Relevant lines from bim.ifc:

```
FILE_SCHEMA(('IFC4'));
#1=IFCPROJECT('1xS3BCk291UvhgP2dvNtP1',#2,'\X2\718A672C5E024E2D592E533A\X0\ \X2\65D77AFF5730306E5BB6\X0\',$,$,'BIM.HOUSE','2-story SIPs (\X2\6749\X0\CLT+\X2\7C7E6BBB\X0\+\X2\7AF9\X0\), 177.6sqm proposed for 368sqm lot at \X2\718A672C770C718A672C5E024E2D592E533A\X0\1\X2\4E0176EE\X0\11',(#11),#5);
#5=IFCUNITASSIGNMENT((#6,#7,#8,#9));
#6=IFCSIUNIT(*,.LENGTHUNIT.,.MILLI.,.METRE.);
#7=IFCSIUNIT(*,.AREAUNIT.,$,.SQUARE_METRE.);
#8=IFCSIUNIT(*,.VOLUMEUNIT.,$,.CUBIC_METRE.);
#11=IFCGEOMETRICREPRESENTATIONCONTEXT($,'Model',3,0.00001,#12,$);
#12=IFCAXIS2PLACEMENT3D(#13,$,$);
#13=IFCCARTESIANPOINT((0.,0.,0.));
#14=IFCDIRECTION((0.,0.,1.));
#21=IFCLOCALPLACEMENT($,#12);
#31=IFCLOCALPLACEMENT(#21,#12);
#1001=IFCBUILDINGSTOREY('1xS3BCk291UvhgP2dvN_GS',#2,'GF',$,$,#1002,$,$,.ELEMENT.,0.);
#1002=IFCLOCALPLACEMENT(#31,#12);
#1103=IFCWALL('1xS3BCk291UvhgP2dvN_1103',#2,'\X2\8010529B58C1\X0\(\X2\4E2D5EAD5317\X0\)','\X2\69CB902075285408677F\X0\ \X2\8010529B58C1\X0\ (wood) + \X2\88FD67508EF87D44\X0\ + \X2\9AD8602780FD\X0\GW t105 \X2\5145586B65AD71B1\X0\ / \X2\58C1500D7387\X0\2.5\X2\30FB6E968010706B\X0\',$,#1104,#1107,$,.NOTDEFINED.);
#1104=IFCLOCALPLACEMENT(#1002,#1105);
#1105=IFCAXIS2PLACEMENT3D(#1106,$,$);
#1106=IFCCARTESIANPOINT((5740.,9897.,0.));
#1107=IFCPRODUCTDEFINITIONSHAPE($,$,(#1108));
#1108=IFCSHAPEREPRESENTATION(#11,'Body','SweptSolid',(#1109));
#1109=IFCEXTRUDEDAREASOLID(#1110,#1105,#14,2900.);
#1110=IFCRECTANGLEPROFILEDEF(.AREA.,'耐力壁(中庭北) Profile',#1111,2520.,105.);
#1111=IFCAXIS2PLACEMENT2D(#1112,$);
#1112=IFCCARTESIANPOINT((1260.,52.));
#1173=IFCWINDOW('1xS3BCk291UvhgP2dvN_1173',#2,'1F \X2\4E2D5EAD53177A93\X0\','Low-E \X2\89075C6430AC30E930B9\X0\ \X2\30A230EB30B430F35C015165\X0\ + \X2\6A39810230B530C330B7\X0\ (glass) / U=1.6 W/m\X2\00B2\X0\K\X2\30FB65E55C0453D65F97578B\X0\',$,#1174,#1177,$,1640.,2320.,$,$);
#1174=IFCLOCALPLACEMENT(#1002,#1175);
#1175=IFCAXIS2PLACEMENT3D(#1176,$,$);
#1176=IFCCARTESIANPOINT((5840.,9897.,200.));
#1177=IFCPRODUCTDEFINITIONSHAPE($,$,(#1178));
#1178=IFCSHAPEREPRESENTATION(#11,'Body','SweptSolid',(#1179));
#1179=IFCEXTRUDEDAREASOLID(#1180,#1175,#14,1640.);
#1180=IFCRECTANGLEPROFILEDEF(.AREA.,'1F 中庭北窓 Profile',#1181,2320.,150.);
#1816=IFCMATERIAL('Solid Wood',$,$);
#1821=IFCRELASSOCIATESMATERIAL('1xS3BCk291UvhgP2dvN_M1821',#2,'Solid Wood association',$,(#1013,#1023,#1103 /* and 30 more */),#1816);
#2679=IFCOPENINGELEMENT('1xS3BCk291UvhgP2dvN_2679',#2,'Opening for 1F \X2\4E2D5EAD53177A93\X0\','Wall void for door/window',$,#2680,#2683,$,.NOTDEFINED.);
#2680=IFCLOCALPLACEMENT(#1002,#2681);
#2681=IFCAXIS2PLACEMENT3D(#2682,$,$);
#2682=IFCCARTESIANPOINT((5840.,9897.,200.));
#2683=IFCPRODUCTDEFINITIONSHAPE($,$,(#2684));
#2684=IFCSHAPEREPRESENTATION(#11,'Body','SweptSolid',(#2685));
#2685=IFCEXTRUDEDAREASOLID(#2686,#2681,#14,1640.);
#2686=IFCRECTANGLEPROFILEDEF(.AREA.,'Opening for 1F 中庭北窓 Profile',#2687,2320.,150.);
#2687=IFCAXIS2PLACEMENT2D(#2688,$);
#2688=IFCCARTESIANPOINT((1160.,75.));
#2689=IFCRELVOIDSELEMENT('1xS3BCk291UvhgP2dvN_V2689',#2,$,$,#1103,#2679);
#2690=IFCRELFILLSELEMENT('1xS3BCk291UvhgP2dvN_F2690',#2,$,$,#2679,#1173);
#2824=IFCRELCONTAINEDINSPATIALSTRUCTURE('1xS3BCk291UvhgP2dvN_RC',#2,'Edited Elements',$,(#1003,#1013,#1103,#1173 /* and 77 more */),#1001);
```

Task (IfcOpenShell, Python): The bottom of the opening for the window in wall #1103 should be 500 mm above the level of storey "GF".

```python
import numpy as np
import ifcopenshell
import ifcopenshell.api.geometry
import ifcopenshell.geom
import ifcopenshell.util.element
import ifcopenshell.util.placement
import ifcopenshell.util.shape
import ifcopenshell.util.unit

model = ifcopenshell.open("bim.ifc")
unit_scale = ifcopenshell.util.unit.calculate_unit_scale(model)

window = model.by_id(1173)
opening = window.FillsVoids[0].RelatingOpeningElement
storey = ifcopenshell.util.element.get_container(window, ifc_class="IfcBuildingStorey")
level = ifcopenshell.util.placement.get_local_placement(storey.ObjectPlacement)[2, 3]

# The opening's origin need not be at the sill, so measure its lowest point.
shape = ifcopenshell.geom.create_shape(ifcopenshell.geom.settings(), opening)
bottom = ifcopenshell.util.shape.get_shape_bottom_elevation(shape, shape.geometry) / unit_scale
dz = level + 0.5 / unit_scale - bottom

shift = np.array([0.0, 0.0, dz])
# The window is not placed relative to its opening, so move both.
for product in (opening, window):
    matrix = ifcopenshell.util.placement.get_local_placement(product.ObjectPlacement)
    matrix[:3, 3] += shift
    ifcopenshell.api.geometry.edit_object_placement(model, product=product, matrix=matrix, is_si=False)

print(f"moved by {dz * unit_scale:+.3f} m")

model.write("bim-out.ifc")
```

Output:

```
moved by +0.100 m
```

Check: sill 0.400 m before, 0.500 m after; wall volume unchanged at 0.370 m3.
